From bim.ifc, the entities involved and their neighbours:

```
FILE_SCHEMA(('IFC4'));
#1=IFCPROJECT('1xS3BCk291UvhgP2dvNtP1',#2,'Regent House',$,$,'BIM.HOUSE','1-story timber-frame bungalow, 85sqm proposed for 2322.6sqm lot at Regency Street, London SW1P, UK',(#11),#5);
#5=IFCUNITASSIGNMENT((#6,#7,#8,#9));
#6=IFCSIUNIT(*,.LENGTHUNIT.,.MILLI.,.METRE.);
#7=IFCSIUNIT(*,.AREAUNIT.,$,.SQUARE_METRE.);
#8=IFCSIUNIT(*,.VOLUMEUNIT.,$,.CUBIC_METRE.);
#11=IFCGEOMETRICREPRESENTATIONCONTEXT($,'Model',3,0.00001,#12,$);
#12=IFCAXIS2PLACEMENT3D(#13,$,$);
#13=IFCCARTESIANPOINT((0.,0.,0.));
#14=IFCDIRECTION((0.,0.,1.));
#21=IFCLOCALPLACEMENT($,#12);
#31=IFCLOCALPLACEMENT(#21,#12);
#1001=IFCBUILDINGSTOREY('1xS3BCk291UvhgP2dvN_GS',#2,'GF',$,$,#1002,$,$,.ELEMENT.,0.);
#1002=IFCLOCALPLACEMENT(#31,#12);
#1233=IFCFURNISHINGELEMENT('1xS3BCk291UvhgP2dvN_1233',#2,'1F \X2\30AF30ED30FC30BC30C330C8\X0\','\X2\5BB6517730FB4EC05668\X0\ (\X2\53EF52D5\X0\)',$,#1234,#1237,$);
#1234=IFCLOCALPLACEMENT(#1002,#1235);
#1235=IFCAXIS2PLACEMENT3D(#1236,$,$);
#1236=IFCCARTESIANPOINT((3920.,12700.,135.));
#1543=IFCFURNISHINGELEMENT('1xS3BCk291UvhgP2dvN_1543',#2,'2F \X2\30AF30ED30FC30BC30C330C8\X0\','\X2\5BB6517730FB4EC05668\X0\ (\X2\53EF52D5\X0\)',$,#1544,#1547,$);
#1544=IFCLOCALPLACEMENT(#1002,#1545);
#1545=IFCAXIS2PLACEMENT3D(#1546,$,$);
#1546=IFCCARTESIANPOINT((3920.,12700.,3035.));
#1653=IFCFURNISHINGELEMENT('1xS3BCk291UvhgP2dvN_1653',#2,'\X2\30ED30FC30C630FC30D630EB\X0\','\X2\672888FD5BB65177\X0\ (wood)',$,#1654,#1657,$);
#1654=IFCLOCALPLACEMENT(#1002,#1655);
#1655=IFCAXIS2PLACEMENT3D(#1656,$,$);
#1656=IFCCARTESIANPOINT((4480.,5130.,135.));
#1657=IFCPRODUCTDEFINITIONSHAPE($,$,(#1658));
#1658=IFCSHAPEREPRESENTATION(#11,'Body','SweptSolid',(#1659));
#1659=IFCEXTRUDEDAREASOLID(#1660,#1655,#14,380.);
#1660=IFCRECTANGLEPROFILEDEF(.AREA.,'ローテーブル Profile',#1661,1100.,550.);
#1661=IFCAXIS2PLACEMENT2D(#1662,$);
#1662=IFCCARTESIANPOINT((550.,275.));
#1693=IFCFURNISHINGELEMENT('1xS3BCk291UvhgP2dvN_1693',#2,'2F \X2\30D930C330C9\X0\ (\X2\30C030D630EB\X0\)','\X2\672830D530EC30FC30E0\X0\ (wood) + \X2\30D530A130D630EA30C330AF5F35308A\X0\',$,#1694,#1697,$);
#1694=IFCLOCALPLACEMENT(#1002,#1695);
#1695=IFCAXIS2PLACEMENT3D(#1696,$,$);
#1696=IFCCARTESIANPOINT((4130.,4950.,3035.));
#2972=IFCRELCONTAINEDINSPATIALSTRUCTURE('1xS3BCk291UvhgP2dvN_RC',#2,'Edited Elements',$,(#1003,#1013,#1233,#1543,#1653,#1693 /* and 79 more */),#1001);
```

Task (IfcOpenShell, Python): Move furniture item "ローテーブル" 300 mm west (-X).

```python
import ifcopenshell
import ifcopenshell.api.geometry
import ifcopenshell.util.placement

model = ifcopenshell.open("bim.ifc")

item = model.by_id(1653)
matrix = ifcopenshell.util.placement.get_local_placement(item.ObjectPlacement)
matrix[0, 3] -= 300.0
ifcopenshell.api.geometry.edit_object_placement(model, product=item, matrix=matrix, is_si=False)

print(ifcopenshell.util.placement.get_local_placement(item.ObjectPlacement).round(3) + 0.0)

model.write("bim-out.ifc")
```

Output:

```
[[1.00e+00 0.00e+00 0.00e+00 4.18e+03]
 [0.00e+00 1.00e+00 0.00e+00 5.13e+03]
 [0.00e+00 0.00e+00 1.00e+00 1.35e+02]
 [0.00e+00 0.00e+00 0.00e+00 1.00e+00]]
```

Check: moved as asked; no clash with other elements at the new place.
